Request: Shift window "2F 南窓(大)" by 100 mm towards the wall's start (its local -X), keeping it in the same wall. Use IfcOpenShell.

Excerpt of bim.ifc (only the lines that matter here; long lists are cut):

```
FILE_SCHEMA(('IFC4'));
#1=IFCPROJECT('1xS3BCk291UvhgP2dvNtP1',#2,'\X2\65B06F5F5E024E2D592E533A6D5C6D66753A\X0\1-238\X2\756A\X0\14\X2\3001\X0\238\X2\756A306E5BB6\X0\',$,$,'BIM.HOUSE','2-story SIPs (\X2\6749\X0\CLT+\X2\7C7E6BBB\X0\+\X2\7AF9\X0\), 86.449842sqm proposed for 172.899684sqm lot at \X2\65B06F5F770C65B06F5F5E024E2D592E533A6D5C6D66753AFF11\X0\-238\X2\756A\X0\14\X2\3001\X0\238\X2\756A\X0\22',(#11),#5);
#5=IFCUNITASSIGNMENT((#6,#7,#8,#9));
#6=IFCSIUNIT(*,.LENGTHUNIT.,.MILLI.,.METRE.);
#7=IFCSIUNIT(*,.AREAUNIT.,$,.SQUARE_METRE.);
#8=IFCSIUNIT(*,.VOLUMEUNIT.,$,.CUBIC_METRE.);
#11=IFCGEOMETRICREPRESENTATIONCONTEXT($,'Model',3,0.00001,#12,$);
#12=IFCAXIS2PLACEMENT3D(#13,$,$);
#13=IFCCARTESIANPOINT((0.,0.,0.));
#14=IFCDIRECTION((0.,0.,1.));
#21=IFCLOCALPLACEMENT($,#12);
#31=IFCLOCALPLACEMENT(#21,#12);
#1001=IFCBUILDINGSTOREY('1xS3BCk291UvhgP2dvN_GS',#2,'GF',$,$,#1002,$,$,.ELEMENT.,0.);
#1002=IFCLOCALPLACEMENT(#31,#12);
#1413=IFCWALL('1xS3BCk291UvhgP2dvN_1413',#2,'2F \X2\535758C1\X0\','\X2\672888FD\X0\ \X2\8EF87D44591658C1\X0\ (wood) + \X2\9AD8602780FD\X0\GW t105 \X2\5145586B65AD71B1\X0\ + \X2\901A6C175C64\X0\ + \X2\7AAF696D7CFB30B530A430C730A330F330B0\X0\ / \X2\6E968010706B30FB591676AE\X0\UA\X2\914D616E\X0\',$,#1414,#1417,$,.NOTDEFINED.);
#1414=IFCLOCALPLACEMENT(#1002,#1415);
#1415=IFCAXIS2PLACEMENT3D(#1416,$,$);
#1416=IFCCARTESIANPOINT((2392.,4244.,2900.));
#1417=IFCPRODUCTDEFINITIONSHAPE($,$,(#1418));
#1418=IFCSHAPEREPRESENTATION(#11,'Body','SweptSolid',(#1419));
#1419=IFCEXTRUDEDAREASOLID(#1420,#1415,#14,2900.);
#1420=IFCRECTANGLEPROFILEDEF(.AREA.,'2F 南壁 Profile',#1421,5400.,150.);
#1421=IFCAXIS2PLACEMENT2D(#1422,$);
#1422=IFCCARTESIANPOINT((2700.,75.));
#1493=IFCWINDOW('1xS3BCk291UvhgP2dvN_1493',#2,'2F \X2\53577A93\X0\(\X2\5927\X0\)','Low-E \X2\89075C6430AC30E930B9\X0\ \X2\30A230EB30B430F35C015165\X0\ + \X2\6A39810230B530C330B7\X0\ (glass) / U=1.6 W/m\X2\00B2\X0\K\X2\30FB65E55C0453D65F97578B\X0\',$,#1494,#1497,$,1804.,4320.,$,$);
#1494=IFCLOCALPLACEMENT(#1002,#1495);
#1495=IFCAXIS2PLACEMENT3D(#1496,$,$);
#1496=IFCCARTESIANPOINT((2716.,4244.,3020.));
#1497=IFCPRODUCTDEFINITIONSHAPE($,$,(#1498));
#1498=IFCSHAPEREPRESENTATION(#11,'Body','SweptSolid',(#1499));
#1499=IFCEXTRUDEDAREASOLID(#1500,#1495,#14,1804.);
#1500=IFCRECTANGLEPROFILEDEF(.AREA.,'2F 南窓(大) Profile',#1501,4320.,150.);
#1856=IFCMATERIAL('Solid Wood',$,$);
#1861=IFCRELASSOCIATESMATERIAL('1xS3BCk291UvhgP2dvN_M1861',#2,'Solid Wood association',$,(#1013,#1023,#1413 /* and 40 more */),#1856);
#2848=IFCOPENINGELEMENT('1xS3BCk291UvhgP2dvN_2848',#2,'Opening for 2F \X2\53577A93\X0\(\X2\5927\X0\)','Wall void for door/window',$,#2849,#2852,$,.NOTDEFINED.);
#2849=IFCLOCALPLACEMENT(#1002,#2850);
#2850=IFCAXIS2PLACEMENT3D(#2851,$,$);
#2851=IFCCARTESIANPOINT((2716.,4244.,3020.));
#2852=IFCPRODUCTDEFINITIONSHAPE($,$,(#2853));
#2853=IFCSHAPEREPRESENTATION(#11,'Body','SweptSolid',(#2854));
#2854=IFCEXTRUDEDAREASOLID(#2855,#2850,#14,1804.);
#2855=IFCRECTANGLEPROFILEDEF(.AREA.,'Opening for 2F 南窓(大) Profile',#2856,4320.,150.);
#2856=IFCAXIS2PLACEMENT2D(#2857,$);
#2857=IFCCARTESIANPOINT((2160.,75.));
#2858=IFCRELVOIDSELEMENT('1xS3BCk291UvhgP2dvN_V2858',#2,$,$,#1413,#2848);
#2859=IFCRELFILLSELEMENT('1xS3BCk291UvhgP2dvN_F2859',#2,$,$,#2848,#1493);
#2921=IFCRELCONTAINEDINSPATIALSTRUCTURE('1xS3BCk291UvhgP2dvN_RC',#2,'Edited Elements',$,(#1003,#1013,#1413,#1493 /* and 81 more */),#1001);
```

```python
import ifcopenshell
import ifcopenshell.api.geometry
import ifcopenshell.util.placement

model = ifcopenshell.open("bim.ifc")

window = model.by_guid("1xS3BCk291UvhgP2dvN_1493")
opening = window.FillsVoids[0].RelatingOpeningElement
wall = opening.VoidsElements[0].RelatingBuildingElement

wall_matrix = ifcopenshell.util.placement.get_local_placement(wall.ObjectPlacement)
shift = wall_matrix[:3, 0] * -100.0
before = ifcopenshell.util.placement.get_local_placement(window.ObjectPlacement)[:3, 3].copy()

# The window is not placed relative to its opening, so move both.
for product in (opening, window):
    matrix = ifcopenshell.util.placement.get_local_placement(product.ObjectPlacement)
    matrix[:3, 3] += shift
    ifcopenshell.api.geometry.edit_object_placement(model, product=product, matrix=matrix, is_si=False)

after = ifcopenshell.util.placement.get_local_placement(window.ObjectPlacement)[:3, 3]
print("window moved by", (after - before).round(3) + 0.0)

model.write("bim_rev.ifc")
```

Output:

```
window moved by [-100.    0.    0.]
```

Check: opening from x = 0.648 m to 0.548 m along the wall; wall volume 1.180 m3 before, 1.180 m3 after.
